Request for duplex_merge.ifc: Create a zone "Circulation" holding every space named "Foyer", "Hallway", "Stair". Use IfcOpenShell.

First a look at what the model holds.

```python
import ifcopenshell

model = ifcopenshell.open("duplex_merge.ifc")
print(model.schema)
seen = {}
for space in model.by_type("IfcSpace"):
    seen[space.LongName] = seen.get(space.LongName, 0) + 1
for name, count in sorted(seen.items(), key=str):
    print(count, "x", name)
print("zones:", [z.Name for z in model.by_type("IfcZone")][:20])
```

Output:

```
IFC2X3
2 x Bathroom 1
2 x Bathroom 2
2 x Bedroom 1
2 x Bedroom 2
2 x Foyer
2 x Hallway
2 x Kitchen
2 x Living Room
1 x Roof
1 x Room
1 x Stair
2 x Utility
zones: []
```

```python
import ifcopenshell
import ifcopenshell.api.group
import ifcopenshell.api.root

model = ifcopenshell.open("duplex_merge.ifc")

names = {"Foyer", "Hallway", "Stair"}
spaces = [s for s in model.by_type("IfcSpace") if s.LongName in names]

zone = ifcopenshell.api.root.create_entity(model, ifc_class="IfcZone", name="Circulation")
ifcopenshell.api.group.assign_group(model, products=spaces, group=zone)
print(len(spaces), "spaces in", zone.Name)

model.write("duplex_merge-out.ifc")
```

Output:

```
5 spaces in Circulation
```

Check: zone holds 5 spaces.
